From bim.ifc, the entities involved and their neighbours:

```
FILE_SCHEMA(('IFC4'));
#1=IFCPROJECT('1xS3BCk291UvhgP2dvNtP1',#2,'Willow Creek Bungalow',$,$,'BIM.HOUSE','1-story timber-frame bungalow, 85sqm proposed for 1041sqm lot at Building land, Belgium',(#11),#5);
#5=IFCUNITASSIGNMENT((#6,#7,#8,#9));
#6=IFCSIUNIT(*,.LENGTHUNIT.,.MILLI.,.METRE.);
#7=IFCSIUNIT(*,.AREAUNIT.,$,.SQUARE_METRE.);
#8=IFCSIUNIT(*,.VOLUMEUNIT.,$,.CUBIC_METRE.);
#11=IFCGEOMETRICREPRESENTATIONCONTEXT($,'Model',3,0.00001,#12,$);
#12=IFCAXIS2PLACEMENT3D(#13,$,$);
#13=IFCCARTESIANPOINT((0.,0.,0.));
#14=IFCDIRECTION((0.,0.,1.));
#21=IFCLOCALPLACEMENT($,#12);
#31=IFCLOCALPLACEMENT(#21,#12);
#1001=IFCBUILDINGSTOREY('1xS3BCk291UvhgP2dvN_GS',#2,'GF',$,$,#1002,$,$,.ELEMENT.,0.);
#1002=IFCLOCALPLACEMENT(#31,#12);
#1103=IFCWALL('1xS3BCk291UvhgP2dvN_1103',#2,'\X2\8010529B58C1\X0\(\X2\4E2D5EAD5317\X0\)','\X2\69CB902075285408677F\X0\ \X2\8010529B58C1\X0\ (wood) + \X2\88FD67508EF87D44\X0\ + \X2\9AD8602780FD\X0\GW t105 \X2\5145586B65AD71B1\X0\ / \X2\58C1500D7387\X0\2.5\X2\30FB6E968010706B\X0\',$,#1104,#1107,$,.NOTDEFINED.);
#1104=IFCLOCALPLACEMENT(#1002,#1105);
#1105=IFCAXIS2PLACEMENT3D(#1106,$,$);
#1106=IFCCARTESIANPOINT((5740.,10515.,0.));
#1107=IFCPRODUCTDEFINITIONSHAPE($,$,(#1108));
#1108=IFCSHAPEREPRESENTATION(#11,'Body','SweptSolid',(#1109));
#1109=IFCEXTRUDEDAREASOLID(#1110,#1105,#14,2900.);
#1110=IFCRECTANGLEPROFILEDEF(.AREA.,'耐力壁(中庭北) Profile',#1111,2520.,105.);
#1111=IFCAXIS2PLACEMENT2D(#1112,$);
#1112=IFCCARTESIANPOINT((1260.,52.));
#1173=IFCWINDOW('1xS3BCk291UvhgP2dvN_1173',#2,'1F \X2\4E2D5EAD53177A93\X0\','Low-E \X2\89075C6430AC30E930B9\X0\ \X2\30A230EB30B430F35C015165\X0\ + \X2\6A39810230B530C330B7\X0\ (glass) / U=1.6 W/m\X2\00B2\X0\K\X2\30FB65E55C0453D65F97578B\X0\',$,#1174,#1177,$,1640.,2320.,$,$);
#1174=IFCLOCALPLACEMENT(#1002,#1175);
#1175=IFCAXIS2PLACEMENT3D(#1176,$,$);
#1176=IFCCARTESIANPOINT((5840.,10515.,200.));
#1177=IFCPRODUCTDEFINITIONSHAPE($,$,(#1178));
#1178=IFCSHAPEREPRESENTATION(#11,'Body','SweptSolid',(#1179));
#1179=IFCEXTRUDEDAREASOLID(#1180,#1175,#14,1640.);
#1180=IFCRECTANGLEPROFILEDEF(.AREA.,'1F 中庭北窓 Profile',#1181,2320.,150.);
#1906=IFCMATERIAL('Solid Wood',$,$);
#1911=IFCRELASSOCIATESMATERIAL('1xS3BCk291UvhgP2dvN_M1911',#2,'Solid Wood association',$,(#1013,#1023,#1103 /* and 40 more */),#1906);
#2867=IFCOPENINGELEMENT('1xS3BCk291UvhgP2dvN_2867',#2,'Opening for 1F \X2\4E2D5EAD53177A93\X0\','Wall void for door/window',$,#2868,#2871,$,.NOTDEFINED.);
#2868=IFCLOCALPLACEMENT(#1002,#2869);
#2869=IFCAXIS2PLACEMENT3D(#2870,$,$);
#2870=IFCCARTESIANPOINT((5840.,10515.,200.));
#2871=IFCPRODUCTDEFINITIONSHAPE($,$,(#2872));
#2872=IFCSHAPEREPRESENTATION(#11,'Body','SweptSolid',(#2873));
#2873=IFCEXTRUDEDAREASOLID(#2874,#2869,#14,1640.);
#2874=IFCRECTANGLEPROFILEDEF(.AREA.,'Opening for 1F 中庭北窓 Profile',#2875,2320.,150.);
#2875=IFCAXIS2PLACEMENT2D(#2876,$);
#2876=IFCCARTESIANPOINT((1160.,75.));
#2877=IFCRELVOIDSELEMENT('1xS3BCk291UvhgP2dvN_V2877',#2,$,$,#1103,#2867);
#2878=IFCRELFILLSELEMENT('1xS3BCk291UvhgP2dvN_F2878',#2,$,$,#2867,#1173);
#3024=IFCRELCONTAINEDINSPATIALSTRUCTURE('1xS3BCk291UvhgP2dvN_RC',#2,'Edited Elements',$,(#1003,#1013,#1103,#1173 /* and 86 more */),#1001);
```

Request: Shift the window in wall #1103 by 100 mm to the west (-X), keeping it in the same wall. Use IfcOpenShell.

```python
import ifcopenshell
import ifcopenshell.api.geometry
import ifcopenshell.util.placement
import ifcopenshell.util.unit

model = ifcopenshell.open("bim.ifc")
unit_scale = ifcopenshell.util.unit.calculate_unit_scale(model)

window = model.by_guid("1xS3BCk291UvhgP2dvN_1173")
opening = window.FillsVoids[0].RelatingOpeningElement
wall = opening.VoidsElements[0].RelatingBuildingElement

wall_matrix = ifcopenshell.util.placement.get_local_placement(wall.ObjectPlacement)
shift = wall_matrix[:3, 0] * -0.1 / unit_scale
before = ifcopenshell.util.placement.get_local_placement(window.ObjectPlacement)[:3, 3].copy()

# The window is not placed relative to its opening, so move both.
for product in (opening, window):
    matrix = ifcopenshell.util.placement.get_local_placement(product.ObjectPlacement)
    matrix[:3, 3] += shift
    ifcopenshell.api.geometry.edit_object_placement(model, product=product, matrix=matrix, is_si=False)

after = ifcopenshell.util.placement.get_local_placement(window.ObjectPlacement)[:3, 3]
print("window moved by", (after - before).round(3) + 0.0)

model.write("bim_v2.ifc")
```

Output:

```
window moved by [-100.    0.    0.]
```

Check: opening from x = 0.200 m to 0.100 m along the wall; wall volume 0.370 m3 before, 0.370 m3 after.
